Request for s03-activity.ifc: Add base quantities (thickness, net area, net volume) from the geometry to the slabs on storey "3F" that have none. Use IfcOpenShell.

First a look at what the model holds.

```python
import ifcopenshell
import ifcopenshell.util.element
import ifcopenshell.util.unit

model = ifcopenshell.open("s03-activity.ifc")
print(model.schema)
for unit_type in ("LENGTHUNIT", "AREAUNIT", "VOLUMEUNIT"):
    print(unit_type, ifcopenshell.util.unit.calculate_unit_scale(model, unit_type))
storey = next(s for s in model.by_type("IfcBuildingStorey") if s.Name == "3F")
slabs = [e for e in ifcopenshell.util.element.get_decomposition(storey) if e.is_a("IfcSlab")]
for e in sorted(slabs, key=lambda e: e.id()):
    print(e.id(), e.is_a(), e.Name, list(ifcopenshell.util.element.get_psets(e, qtos_only=True)), sep=" | ")
```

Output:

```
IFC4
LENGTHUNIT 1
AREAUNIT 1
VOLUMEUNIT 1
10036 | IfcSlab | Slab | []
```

```python
import ifcopenshell
import ifcopenshell.api.pset
import ifcopenshell.geom
import ifcopenshell.util.element
import ifcopenshell.util.shape
import ifcopenshell.util.unit

model = ifcopenshell.open("s03-activity.ifc")
unit_scale = ifcopenshell.util.unit.calculate_unit_scale(model)
area_scale = ifcopenshell.util.unit.calculate_unit_scale(model, "AREAUNIT")
volume_scale = ifcopenshell.util.unit.calculate_unit_scale(model, "VOLUMEUNIT")
settings = ifcopenshell.geom.settings()

storey = next(s for s in model.by_type("IfcBuildingStorey") if s.Name == "3F")
slabs = [e for e in ifcopenshell.util.element.get_decomposition(storey) if e.is_a("IfcSlab")]

for e in sorted(slabs, key=lambda e: e.id()):
    if ifcopenshell.util.element.get_psets(e, qtos_only=True, should_inherit=False):
        continue
    # Geometry comes back in metres, in the element's own axes.
    shape = ifcopenshell.geom.create_shape(settings, e)
    values = {
        "Width": ifcopenshell.util.shape.get_z(shape.geometry) / unit_scale,
        "NetArea": ifcopenshell.util.shape.get_footprint_area(shape.geometry) / area_scale,
        "NetVolume": ifcopenshell.util.shape.get_volume(shape.geometry) / volume_scale,
    }
    qto = ifcopenshell.api.pset.add_qto(model, product=e, name="Qto_SlabBaseQuantities")
    ifcopenshell.api.pset.edit_qto(model, qto=qto, properties=values)
    print(e.id(), {k: round(v, 3) for k, v in values.items()})

model.write("s03-activity_rev.ifc")
```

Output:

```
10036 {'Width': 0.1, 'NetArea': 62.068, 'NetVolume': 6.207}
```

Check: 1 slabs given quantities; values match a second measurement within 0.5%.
